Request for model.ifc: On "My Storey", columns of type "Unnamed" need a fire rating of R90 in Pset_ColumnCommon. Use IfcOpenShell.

First a look at what the model holds.

```python
import ifcopenshell
import ifcopenshell.util.element

model = ifcopenshell.open("model.ifc")
print(model.schema)
storey = next(s for s in model.by_type("IfcBuildingStorey") if s.Name == "My Storey")
columns = [e for e in ifcopenshell.util.element.get_decomposition(storey) if e.is_a("IfcColumn")]
seen = {}
for e in columns:
    element_type = ifcopenshell.util.element.get_type(e)
    key = (element_type.Name if element_type != e and element_type else None, ifcopenshell.util.element.get_pset(e, "Pset_ColumnCommon", "FireRating"))
    seen[key] = seen.get(key, 0) + 1
for (name, value), count in sorted(seen.items(), key=str):
    print(count, "x", name, "|", value)
```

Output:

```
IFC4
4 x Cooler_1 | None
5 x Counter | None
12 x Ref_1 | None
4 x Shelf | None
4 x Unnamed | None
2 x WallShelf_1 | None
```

```python
import ifcopenshell
import ifcopenshell.api.pset
import ifcopenshell.util.element

model = ifcopenshell.open("model.ifc")

storey = next(s for s in model.by_type("IfcBuildingStorey") if s.Name == "My Storey")
columns = [e for e in ifcopenshell.util.element.get_decomposition(storey) if e.is_a("IfcColumn")]

count = 0
for e in columns:
    element_type = ifcopenshell.util.element.get_type(e)
    if element_type in (None, e) or element_type.Name != "Unnamed":
        continue
    # add_pset returns the element's existing set when there is one.
    pset = ifcopenshell.api.pset.add_pset(model, product=e, name="Pset_ColumnCommon")
    ifcopenshell.api.pset.edit_pset(model, pset=pset, properties={"FireRating": "R90"})
    count += 1

print(count, "columns updated")

model.write("model_edited.ifc")
```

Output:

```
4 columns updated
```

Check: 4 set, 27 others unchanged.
